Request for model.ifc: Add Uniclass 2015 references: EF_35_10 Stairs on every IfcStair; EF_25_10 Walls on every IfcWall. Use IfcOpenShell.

First a look at what the model holds.

```python
import ifcopenshell

model = ifcopenshell.open("model.ifc")
print(model.schema)
print("classifications:", [c.Name for c in model.by_type("IfcClassification")])
for ifc_class in ("IfcDoor", "IfcRoof", "IfcStair", "IfcWall", "IfcWindow"):
    print(ifc_class, len(model.by_type(ifc_class)))
```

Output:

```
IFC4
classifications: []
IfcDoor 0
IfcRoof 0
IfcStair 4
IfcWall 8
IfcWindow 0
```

```python
import ifcopenshell
import ifcopenshell.api.classification

model = ifcopenshell.open("model.ifc")

system = ifcopenshell.api.classification.add_classification(model, classification="Uniclass 2015")

codes = {
    "IfcStair": ("EF_35_10", "Stairs"),
    "IfcWall": ("EF_25_10", "Walls"),
}
for ifc_class, (code, name) in codes.items():
    products = model.by_type(ifc_class)
    ifcopenshell.api.classification.add_reference(
        model, products=products, classification=system, identification=code, name=name
    )
    print(code, len(products))

model.write("model_edited.ifc")
```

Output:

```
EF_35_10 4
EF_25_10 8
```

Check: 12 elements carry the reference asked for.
